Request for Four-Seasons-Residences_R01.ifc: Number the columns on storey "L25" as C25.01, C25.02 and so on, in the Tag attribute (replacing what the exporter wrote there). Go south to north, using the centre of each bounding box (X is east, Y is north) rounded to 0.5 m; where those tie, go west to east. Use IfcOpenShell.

First a look at what the model holds.

```python
import ifcopenshell
import ifcopenshell.util.element
import ifcopenshell.util.placement

model = ifcopenshell.open("Four-Seasons-Residences_R01.ifc")
print(model.schema)
storey = next(s for s in model.by_type("IfcBuildingStorey") if s.Name == "L25")
columns = [e for e in ifcopenshell.util.element.get_decomposition(storey) if e.is_a("IfcColumn")]
for e in sorted(columns, key=lambda e: e.id()):
    origin = ifcopenshell.util.placement.get_local_placement(e.ObjectPlacement)[:3, 3]
    print(e.id(), e.Tag, e.Name, origin.round(2) + 0.0, sep=" | ")
```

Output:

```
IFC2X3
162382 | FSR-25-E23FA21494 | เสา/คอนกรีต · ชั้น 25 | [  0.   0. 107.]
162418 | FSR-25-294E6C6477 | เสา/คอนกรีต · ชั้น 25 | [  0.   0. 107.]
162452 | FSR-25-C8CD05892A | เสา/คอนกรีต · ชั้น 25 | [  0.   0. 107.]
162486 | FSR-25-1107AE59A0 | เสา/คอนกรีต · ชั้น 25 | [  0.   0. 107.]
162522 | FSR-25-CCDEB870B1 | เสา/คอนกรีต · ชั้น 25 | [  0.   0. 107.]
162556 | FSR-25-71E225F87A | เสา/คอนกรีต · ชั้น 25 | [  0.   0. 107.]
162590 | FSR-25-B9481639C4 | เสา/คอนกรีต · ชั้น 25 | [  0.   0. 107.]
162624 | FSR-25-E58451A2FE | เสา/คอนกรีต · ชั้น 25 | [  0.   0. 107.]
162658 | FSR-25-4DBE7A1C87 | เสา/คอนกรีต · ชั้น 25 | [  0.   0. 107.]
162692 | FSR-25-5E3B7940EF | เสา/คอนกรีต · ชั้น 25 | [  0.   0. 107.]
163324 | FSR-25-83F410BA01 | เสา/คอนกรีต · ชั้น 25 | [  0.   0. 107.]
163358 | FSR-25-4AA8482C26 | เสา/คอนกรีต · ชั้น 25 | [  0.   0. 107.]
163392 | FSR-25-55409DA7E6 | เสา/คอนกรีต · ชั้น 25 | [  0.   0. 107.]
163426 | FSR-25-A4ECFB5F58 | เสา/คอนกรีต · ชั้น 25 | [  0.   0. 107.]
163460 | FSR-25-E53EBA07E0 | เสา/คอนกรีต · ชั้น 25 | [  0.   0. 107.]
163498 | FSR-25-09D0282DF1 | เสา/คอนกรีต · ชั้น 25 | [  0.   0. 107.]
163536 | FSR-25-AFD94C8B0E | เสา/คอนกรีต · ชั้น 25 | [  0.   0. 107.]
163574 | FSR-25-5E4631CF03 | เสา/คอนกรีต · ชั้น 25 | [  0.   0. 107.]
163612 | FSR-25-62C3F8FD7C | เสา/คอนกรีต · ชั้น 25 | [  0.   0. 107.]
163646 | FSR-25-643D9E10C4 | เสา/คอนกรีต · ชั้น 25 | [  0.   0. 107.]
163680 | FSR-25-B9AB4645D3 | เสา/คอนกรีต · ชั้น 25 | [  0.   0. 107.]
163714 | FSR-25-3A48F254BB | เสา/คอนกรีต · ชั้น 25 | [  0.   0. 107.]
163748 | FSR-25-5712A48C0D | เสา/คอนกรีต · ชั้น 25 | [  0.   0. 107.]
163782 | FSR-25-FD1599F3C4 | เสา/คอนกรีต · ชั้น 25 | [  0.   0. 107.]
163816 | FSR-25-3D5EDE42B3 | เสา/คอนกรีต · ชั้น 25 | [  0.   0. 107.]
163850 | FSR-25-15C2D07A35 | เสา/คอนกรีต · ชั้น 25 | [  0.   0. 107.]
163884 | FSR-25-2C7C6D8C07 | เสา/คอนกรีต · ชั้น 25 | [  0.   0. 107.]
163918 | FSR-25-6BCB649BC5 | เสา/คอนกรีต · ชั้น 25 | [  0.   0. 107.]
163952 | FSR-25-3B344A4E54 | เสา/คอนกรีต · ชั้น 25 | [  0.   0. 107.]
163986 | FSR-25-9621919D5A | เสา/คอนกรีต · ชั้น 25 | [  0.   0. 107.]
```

```python
import ifcopenshell
import ifcopenshell.geom
import ifcopenshell.util.element
import ifcopenshell.util.shape

model = ifcopenshell.open("Four-Seasons-Residences_R01.ifc")
settings = ifcopenshell.geom.settings()
settings.set("use-world-coords", True)


def centre(element):
    shape = ifcopenshell.geom.create_shape(settings, element)
    return ifcopenshell.util.shape.get_bbox_centroid(shape.geometry)


storey = next(s for s in model.by_type("IfcBuildingStorey") if s.Name == "L25")
columns = [e for e in ifcopenshell.util.element.get_decomposition(storey) if e.is_a("IfcColumn")]

# Insertion points can sit at a corner or the storey origin, so sort by the geometry (in metres).
centres = {e: centre(e) for e in columns}
columns.sort(key=lambda e: (round(centres[e][1] / 0.5), centres[e][0]))

for i, e in enumerate(columns, start=1):
    number = f"C25.{i:02d}"
    e.Tag = number
    print(e.id(), number)

model.write("Four-Seasons-Residences_R01-out.ifc")
```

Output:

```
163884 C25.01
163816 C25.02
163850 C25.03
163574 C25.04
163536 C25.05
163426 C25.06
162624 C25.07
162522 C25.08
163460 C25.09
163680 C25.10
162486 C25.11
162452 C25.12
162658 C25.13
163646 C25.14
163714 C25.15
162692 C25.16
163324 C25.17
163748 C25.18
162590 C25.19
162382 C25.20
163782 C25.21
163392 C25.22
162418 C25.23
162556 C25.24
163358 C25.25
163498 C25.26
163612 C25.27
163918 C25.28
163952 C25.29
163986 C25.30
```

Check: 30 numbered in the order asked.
